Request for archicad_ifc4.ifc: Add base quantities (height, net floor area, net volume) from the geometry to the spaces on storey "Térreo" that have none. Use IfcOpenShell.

First a look at what the model holds.

```python
import ifcopenshell
import ifcopenshell.util.element
import ifcopenshell.util.unit

model = ifcopenshell.open("archicad_ifc4.ifc")
print(model.schema)
for unit_type in ("LENGTHUNIT", "AREAUNIT", "VOLUMEUNIT"):
    print(unit_type, ifcopenshell.util.unit.calculate_unit_scale(model, unit_type))
storey = next(s for s in model.by_type("IfcBuildingStorey") if s.Name == "Térreo")
spaces = [e for e in ifcopenshell.util.element.get_decomposition(storey) if e.is_a("IfcSpace")]
for e in sorted(spaces, key=lambda e: e.id()):
    print(e.id(), e.is_a(), e.Name, list(ifcopenshell.util.element.get_psets(e, qtos_only=True)), sep=" | ")
```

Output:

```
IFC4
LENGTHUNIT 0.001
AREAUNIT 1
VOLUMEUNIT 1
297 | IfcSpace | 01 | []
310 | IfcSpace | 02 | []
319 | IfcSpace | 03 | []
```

```python
import ifcopenshell
import ifcopenshell.api.pset
import ifcopenshell.geom
import ifcopenshell.util.element
import ifcopenshell.util.shape
import ifcopenshell.util.unit

model = ifcopenshell.open("archicad_ifc4.ifc")
unit_scale = ifcopenshell.util.unit.calculate_unit_scale(model)
area_scale = ifcopenshell.util.unit.calculate_unit_scale(model, "AREAUNIT")
volume_scale = ifcopenshell.util.unit.calculate_unit_scale(model, "VOLUMEUNIT")
settings = ifcopenshell.geom.settings()

storey = next(s for s in model.by_type("IfcBuildingStorey") if s.Name == "Térreo")
spaces = [e for e in ifcopenshell.util.element.get_decomposition(storey) if e.is_a("IfcSpace")]

for e in sorted(spaces, key=lambda e: e.id()):
    if ifcopenshell.util.element.get_psets(e, qtos_only=True, should_inherit=False):
        continue
    # Geometry comes back in metres, in the element's own axes.
    shape = ifcopenshell.geom.create_shape(settings, e)
    values = {
        "Height": ifcopenshell.util.shape.get_z(shape.geometry) / unit_scale,
        "NetFloorArea": ifcopenshell.util.shape.get_footprint_area(shape.geometry) / area_scale,
        "NetVolume": ifcopenshell.util.shape.get_volume(shape.geometry) / volume_scale,
    }
    qto = ifcopenshell.api.pset.add_qto(model, product=e, name="Qto_SpaceBaseQuantities")
    ifcopenshell.api.pset.edit_qto(model, qto=qto, properties=values)
    print(e.id(), {k: round(v, 3) for k, v in values.items()})

model.write("archicad_ifc4_rev.ifc")
```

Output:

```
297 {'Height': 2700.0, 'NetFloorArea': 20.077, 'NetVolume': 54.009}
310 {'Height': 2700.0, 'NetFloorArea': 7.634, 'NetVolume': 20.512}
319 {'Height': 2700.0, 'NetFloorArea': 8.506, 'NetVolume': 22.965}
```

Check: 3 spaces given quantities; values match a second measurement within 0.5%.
